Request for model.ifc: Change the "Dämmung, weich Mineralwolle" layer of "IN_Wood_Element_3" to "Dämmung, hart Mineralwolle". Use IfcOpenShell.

First a look at what the model holds.

```python
import ifcopenshell
import ifcopenshell.util.element

model = ifcopenshell.open("model.ifc")
print(model.schema)
for layer_set in model.by_type("IfcMaterialLayerSet"):
    if layer_set.LayerSetName == "IN_Wood_Element_3":
        for layer in layer_set.MaterialLayers:
            print(layer.id(), layer.Material and layer.Material.Name, layer.LayerThickness, sep=" | ")
        print(len(ifcopenshell.util.element.get_elements_by_material(model, layer_set)), "elements and types use it")
print(sorted(m.Name for m in model.by_type("IfcMaterial") if m.Name)[:60])
```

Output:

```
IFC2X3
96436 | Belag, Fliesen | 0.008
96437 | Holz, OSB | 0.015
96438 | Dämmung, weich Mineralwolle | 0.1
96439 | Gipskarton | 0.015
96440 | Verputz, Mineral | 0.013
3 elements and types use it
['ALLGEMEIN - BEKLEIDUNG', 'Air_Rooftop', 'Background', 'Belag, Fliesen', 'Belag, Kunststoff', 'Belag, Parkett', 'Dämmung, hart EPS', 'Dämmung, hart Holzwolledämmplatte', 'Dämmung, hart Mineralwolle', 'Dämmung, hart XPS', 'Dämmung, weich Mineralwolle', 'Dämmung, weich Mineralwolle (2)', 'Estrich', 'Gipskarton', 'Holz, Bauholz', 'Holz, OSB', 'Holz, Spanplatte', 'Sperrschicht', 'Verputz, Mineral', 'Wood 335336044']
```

```python
import ifcopenshell
import ifcopenshell.api.material

model = ifcopenshell.open("model.ifc")

layer_set = next(s for s in model.by_type("IfcMaterialLayerSet") if s.LayerSetName == "IN_Wood_Element_3")
layer = next(l for l in layer_set.MaterialLayers if l.Material and l.Material.Name == "Dämmung, weich Mineralwolle")
material = next(m for m in model.by_type("IfcMaterial") if m.Name == "Dämmung, hart Mineralwolle")

# Point this one layer at the other material; renaming the old one would change it everywhere.
ifcopenshell.api.material.edit_layer(model, layer=layer, attributes={}, material=material)

print([l.Material.Name if l.Material else None for l in layer_set.MaterialLayers])

model.write("model_v2.ifc")
```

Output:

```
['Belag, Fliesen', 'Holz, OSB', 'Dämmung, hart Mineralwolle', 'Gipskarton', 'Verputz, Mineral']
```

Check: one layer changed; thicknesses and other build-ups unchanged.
